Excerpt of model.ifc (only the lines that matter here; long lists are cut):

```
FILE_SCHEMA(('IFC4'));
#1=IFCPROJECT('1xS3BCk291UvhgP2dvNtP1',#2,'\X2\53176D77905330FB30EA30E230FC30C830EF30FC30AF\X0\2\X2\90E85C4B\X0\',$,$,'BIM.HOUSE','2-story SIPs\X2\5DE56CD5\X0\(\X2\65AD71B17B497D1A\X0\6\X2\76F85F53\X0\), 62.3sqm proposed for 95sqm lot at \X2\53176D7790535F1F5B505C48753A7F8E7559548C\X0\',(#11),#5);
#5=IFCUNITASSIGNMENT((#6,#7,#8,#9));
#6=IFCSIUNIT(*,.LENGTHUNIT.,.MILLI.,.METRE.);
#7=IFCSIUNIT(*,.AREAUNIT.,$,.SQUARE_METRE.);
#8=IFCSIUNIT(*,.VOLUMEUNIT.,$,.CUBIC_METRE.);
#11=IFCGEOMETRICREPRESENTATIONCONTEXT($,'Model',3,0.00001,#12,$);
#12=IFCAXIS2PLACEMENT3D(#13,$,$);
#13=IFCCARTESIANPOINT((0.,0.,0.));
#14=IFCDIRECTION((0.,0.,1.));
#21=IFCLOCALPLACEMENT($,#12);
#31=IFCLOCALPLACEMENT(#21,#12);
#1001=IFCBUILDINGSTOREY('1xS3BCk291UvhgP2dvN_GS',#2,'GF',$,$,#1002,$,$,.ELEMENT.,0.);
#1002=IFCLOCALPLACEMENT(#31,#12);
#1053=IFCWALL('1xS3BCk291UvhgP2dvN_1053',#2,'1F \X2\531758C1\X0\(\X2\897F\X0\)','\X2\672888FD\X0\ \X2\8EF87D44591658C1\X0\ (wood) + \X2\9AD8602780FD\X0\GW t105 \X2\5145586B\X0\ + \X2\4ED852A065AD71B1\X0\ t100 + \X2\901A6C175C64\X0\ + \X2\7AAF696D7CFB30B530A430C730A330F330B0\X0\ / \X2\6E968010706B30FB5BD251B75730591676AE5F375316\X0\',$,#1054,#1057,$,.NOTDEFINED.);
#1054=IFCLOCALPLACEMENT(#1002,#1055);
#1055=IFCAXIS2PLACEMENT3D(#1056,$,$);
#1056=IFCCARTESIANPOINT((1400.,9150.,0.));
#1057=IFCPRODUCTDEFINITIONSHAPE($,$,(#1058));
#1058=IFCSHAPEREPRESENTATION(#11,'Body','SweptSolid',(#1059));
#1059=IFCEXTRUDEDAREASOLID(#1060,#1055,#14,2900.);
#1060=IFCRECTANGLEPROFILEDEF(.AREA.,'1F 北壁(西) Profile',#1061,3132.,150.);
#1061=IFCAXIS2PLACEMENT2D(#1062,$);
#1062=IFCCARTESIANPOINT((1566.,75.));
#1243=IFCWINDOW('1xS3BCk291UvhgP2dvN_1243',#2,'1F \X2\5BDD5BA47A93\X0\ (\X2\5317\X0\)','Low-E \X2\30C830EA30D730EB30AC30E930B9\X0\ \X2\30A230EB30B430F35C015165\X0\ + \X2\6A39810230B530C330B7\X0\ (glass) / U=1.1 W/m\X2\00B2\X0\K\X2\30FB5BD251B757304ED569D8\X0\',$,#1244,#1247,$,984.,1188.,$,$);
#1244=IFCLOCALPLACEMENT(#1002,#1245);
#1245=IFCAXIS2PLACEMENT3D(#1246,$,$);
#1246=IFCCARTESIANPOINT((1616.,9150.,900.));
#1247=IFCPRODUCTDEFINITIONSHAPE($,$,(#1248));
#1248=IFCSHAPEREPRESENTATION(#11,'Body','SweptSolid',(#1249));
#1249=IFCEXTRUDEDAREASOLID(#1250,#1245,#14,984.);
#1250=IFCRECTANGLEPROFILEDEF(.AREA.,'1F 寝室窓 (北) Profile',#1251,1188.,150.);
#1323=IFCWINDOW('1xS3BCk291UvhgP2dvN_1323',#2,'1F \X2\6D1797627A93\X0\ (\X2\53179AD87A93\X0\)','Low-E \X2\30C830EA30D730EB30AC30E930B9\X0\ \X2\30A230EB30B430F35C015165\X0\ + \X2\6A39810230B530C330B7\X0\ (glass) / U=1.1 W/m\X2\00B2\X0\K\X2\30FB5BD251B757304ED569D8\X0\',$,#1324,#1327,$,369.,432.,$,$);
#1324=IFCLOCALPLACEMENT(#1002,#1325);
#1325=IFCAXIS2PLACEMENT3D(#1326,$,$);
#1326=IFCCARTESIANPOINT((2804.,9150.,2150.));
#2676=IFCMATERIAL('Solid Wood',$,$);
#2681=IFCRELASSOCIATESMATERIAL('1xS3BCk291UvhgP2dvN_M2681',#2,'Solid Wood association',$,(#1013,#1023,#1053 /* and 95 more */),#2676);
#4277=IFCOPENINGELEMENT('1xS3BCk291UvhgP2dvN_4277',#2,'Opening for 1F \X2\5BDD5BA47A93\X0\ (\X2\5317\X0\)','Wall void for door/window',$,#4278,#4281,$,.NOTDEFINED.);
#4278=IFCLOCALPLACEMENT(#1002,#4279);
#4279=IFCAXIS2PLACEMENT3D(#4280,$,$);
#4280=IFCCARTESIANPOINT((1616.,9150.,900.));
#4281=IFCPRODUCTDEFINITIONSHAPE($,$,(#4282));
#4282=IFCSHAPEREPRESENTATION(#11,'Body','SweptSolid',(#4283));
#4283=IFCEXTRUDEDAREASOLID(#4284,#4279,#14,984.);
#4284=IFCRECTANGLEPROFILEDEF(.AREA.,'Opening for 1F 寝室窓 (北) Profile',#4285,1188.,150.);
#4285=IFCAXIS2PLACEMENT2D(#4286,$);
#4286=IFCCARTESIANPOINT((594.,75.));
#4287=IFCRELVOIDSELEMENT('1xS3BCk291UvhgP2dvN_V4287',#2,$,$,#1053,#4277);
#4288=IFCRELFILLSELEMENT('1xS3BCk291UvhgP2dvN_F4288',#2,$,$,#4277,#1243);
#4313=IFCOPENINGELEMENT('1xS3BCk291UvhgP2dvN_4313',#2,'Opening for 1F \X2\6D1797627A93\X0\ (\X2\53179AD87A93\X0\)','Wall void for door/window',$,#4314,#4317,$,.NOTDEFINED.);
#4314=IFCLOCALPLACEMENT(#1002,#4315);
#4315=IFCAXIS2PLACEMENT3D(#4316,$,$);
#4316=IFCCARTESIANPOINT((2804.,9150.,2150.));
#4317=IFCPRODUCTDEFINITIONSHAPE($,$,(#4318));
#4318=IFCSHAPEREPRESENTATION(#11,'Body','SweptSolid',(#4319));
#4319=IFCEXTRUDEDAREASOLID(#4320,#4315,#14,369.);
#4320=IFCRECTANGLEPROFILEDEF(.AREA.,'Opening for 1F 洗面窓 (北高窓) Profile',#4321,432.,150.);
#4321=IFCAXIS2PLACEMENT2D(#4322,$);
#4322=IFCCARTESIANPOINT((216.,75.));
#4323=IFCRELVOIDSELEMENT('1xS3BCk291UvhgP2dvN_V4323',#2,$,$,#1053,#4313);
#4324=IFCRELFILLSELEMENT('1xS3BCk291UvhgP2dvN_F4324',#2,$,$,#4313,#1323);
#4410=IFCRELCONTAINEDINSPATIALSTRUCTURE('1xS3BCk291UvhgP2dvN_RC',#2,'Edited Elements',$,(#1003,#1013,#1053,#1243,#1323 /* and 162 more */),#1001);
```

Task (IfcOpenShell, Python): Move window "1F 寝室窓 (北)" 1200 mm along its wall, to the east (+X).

```python
import ifcopenshell
import ifcopenshell.api.geometry
import ifcopenshell.util.placement
import ifcopenshell.util.unit

model = ifcopenshell.open("model.ifc")
unit_scale = ifcopenshell.util.unit.calculate_unit_scale(model)

window = model.by_guid("1xS3BCk291UvhgP2dvN_1243")
opening = window.FillsVoids[0].RelatingOpeningElement
wall = opening.VoidsElements[0].RelatingBuildingElement

wall_matrix = ifcopenshell.util.placement.get_local_placement(wall.ObjectPlacement)
shift = wall_matrix[:3, 0] * 1.2 / unit_scale
before = ifcopenshell.util.placement.get_local_placement(window.ObjectPlacement)[:3, 3].copy()

# The window is not placed relative to its opening, so move both.
for product in (opening, window):
    matrix = ifcopenshell.util.placement.get_local_placement(product.ObjectPlacement)
    matrix[:3, 3] += shift
    ifcopenshell.api.geometry.edit_object_placement(model, product=product, matrix=matrix, is_si=False)

after = ifcopenshell.util.placement.get_local_placement(window.ObjectPlacement)[:3, 3]
print("window moved by", (after - before).round(3) + 0.0)

model.write("model_v2.ifc")
```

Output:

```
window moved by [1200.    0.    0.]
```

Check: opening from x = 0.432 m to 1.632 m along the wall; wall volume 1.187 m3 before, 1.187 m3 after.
